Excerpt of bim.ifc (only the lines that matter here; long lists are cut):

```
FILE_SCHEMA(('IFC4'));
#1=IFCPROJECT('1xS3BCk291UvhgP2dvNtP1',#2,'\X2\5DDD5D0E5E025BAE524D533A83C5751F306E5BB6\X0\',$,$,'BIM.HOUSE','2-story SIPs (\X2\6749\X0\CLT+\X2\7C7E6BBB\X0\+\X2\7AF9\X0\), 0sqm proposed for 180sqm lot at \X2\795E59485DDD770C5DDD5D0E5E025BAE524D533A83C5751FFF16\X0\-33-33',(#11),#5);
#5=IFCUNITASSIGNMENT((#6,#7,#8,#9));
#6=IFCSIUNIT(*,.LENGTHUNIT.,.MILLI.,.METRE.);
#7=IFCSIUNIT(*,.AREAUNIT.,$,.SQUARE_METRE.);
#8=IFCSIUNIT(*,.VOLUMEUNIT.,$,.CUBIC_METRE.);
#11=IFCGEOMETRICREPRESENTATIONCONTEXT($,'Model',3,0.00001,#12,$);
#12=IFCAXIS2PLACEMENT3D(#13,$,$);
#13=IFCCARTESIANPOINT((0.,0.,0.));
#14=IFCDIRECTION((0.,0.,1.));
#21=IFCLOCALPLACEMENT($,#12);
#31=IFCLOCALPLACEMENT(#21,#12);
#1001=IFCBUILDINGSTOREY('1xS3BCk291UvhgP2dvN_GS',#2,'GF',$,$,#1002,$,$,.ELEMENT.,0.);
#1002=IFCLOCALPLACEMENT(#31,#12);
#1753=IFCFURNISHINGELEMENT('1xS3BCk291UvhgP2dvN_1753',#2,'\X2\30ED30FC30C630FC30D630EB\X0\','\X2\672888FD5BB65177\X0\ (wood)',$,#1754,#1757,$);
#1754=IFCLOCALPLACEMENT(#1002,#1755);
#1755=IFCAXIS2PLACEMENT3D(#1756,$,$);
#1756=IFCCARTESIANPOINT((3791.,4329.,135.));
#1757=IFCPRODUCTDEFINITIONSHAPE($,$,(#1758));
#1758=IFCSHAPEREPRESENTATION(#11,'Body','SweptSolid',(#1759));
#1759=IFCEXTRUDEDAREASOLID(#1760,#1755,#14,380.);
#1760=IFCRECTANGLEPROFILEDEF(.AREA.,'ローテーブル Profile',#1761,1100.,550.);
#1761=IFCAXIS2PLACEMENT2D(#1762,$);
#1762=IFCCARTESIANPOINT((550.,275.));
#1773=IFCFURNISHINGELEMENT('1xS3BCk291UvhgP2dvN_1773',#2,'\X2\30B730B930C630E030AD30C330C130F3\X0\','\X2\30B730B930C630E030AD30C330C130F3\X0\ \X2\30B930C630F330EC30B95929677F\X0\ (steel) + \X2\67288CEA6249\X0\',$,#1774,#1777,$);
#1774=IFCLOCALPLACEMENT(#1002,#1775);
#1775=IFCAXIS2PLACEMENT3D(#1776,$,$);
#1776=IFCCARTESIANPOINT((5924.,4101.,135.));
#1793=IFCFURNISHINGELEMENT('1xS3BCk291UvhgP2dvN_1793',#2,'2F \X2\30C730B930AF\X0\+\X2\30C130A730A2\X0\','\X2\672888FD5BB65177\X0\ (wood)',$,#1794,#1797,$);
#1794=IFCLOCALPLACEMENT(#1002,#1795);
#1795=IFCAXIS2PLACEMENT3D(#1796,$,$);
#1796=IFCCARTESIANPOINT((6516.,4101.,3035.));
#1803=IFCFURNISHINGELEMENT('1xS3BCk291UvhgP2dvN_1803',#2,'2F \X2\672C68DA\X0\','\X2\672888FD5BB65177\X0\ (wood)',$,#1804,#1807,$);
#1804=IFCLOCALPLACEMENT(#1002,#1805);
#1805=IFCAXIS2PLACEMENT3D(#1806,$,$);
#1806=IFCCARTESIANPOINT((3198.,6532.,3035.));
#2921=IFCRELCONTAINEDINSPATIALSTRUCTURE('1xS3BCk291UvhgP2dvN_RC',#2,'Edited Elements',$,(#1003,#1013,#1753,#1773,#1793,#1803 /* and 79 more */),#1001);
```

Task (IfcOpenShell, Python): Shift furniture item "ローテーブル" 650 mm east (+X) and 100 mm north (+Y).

```python
import ifcopenshell
import ifcopenshell.api.geometry
import ifcopenshell.util.placement

model = ifcopenshell.open("bim.ifc")

item = model.by_guid("1xS3BCk291UvhgP2dvN_1753")
matrix = ifcopenshell.util.placement.get_local_placement(item.ObjectPlacement)
matrix[0, 3] += 650.0
matrix[1, 3] += 100.0
ifcopenshell.api.geometry.edit_object_placement(model, product=item, matrix=matrix, is_si=False)

print(ifcopenshell.util.placement.get_local_placement(item.ObjectPlacement).round(3) + 0.0)

model.write("bim_rev.ifc")
```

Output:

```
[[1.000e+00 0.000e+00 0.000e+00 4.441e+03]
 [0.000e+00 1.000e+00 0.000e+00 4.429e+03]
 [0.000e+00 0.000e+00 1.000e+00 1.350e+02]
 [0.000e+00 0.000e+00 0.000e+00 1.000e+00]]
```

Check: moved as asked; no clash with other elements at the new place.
